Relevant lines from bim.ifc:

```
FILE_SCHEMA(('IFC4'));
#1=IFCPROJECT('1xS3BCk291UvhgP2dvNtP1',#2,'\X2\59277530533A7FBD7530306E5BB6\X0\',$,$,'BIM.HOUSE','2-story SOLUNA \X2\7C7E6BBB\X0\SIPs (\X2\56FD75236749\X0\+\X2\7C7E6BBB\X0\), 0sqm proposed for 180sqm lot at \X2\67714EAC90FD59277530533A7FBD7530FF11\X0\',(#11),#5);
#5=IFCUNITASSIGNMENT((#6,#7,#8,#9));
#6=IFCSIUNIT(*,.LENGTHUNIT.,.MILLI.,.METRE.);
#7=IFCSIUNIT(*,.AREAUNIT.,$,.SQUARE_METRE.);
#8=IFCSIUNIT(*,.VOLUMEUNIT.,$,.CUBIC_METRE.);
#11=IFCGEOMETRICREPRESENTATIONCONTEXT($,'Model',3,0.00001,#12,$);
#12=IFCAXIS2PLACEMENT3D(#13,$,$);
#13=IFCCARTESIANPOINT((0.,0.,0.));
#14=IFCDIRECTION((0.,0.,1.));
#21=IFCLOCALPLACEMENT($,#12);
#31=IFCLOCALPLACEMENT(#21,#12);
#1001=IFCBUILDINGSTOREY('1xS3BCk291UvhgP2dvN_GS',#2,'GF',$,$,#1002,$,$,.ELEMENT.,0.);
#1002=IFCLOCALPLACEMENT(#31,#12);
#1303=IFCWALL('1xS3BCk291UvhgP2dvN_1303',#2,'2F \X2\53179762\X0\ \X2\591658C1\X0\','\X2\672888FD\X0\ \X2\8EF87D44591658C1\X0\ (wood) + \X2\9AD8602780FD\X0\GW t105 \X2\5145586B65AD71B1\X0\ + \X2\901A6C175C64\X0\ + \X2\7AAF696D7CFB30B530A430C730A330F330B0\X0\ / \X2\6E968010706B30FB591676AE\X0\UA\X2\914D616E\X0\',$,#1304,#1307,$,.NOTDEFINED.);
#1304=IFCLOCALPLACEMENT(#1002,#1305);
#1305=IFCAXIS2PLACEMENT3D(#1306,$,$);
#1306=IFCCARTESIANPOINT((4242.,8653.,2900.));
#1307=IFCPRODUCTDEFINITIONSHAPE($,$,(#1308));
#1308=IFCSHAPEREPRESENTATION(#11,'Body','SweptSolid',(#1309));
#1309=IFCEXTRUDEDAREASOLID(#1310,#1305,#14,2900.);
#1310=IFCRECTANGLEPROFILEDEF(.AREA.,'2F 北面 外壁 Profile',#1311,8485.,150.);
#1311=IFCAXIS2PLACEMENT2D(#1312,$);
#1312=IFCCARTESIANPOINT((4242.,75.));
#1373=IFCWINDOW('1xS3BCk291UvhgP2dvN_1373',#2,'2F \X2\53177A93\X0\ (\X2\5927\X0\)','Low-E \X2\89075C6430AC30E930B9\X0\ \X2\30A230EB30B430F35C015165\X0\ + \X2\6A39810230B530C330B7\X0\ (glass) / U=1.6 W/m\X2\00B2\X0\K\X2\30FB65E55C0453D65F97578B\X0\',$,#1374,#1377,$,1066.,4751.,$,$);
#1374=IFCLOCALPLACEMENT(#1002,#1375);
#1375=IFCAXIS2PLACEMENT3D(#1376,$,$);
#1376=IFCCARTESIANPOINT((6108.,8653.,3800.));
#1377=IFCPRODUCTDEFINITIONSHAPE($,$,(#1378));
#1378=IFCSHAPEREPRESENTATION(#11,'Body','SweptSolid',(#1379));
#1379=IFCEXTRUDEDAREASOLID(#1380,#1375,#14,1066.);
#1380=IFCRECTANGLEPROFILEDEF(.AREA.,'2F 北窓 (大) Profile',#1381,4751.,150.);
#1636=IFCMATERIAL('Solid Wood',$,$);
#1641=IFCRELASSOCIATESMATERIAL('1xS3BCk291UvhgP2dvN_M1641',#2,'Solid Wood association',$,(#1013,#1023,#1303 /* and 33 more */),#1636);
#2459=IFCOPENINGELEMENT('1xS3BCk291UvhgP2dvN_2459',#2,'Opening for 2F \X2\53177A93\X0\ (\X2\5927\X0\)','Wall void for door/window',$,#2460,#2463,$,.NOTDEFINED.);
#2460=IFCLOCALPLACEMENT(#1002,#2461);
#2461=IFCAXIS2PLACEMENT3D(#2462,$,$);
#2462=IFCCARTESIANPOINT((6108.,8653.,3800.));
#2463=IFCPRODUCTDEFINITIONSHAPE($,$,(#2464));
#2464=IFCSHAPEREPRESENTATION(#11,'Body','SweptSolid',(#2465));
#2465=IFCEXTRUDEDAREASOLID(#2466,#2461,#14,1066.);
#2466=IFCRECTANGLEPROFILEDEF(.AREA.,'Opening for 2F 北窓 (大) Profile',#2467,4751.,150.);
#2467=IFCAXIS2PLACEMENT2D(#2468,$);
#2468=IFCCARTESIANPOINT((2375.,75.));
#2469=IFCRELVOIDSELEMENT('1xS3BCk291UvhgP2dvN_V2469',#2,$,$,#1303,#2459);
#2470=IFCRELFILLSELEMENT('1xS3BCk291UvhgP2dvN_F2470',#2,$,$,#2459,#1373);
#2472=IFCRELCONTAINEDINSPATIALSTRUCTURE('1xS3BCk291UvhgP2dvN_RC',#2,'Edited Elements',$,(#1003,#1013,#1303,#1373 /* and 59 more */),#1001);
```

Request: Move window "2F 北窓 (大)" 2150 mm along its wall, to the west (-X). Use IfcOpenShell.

```python
import ifcopenshell
import ifcopenshell.api.geometry
import ifcopenshell.util.placement

model = ifcopenshell.open("bim.ifc")

window = model.by_id(1373)
opening = window.FillsVoids[0].RelatingOpeningElement
wall = opening.VoidsElements[0].RelatingBuildingElement

wall_matrix = ifcopenshell.util.placement.get_local_placement(wall.ObjectPlacement)
shift = wall_matrix[:3, 0] * -2150.0
before = ifcopenshell.util.placement.get_local_placement(window.ObjectPlacement)[:3, 3].copy()

# The window is not placed relative to its opening, so move both.
for product in (opening, window):
    matrix = ifcopenshell.util.placement.get_local_placement(product.ObjectPlacement)
    matrix[:3, 3] += shift
    ifcopenshell.api.geometry.edit_object_placement(model, product=product, matrix=matrix, is_si=False)

after = ifcopenshell.util.placement.get_local_placement(window.ObjectPlacement)[:3, 3]
print("window moved by", (after - before).round(3) + 0.0)

model.write("bim_v2.ifc")
```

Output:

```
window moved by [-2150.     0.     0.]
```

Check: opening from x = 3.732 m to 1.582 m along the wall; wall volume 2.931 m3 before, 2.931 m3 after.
